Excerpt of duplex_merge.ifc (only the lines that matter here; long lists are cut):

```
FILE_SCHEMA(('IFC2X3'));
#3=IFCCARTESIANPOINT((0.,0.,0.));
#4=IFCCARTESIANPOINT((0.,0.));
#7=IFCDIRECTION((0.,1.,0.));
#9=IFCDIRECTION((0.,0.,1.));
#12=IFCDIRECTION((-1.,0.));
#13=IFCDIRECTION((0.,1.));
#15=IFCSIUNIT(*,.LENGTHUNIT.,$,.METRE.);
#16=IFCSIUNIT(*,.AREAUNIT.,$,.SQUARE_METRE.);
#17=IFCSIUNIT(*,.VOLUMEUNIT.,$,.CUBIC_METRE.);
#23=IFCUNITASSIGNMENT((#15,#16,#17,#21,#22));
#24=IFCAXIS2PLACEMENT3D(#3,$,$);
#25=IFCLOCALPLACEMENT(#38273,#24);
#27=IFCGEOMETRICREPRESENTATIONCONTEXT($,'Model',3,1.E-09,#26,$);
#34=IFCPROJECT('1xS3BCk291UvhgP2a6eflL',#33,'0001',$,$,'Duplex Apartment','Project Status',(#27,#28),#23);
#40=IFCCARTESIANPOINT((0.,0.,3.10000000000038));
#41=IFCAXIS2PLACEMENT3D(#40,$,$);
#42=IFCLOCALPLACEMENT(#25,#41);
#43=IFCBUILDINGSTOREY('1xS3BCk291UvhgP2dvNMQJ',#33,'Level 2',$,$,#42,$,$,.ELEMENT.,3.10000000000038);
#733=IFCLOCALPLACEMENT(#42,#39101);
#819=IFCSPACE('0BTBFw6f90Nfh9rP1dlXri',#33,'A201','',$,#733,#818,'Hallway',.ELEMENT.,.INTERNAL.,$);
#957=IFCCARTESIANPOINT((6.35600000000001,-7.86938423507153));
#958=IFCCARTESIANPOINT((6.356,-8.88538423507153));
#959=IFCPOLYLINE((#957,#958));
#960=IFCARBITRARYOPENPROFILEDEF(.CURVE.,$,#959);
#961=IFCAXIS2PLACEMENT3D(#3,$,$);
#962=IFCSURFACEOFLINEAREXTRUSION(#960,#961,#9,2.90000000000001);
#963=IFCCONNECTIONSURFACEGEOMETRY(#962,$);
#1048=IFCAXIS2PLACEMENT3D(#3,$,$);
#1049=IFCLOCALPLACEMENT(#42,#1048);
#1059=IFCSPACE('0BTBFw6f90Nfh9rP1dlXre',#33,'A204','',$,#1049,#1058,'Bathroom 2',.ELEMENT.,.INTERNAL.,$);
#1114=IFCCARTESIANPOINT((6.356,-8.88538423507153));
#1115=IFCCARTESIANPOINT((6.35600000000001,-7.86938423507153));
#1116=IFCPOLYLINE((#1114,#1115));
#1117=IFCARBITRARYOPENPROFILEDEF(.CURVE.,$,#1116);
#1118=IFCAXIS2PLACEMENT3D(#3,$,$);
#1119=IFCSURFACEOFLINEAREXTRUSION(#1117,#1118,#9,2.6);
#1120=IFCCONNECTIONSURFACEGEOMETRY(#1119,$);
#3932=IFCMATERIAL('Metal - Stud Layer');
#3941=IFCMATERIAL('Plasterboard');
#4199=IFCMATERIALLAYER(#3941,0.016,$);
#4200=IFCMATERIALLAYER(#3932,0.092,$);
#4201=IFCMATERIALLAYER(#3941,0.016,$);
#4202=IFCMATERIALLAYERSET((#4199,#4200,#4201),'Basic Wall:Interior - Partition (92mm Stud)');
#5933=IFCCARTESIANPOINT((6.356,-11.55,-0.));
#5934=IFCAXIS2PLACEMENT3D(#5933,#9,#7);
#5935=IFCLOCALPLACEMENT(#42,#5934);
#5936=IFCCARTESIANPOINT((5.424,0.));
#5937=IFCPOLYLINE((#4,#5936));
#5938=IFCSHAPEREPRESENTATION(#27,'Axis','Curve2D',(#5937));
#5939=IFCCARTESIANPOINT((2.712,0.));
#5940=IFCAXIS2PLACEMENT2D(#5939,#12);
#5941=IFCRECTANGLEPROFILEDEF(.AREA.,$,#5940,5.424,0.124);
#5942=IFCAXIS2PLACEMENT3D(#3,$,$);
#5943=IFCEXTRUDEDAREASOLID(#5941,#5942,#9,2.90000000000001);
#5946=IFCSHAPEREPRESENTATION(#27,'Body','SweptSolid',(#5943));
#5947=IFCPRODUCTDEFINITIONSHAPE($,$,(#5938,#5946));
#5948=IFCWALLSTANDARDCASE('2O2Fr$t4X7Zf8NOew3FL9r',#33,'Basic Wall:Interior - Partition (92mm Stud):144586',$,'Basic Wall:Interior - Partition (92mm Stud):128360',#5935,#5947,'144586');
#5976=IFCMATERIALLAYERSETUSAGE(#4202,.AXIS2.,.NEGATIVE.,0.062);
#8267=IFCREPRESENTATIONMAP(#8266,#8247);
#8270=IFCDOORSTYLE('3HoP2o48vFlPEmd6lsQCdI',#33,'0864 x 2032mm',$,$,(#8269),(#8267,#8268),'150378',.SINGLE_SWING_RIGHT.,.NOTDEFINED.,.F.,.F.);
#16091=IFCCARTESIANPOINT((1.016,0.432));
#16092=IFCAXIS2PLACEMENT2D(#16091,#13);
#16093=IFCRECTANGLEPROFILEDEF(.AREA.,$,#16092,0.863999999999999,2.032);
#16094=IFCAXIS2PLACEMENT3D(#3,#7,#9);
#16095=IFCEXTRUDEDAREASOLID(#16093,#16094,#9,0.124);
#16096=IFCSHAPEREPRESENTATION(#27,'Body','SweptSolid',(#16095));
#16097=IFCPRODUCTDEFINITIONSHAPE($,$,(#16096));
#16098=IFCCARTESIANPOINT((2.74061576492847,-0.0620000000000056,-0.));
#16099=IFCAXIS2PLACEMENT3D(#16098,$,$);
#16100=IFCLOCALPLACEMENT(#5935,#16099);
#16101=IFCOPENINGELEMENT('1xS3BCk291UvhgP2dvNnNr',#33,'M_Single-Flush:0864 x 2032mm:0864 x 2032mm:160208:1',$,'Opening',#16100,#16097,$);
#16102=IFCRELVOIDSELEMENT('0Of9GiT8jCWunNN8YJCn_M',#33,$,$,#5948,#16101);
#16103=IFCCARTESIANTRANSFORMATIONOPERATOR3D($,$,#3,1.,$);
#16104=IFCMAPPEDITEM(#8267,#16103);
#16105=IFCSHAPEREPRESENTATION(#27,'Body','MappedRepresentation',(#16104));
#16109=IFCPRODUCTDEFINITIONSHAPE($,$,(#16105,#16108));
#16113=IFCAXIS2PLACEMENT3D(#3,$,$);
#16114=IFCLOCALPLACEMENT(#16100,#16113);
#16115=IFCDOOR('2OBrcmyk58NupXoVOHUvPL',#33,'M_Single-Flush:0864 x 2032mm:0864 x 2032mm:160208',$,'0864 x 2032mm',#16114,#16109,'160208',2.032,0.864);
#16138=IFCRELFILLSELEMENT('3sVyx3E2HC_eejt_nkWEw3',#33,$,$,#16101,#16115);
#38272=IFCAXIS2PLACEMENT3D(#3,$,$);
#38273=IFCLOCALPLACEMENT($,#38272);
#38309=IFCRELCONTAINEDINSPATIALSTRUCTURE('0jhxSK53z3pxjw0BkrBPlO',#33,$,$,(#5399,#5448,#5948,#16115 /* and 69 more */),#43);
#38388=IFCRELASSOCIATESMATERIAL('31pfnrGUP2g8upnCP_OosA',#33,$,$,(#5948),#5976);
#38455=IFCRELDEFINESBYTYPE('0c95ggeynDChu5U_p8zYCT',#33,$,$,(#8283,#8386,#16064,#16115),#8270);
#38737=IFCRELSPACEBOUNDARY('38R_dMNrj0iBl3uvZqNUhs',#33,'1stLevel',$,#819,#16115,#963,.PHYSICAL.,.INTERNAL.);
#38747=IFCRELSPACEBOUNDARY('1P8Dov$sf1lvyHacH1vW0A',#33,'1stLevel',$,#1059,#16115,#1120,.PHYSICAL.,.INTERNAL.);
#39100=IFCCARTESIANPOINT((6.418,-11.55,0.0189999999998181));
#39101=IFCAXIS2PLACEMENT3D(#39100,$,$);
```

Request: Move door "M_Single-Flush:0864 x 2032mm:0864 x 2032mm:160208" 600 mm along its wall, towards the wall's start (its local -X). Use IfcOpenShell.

```python
import numpy as np
import ifcopenshell
import ifcopenshell.api.geometry
import ifcopenshell.util.placement

model = ifcopenshell.open("duplex_merge.ifc")

door = model.by_id(16115)
opening = door.FillsVoids[0].RelatingOpeningElement
wall = opening.VoidsElements[0].RelatingBuildingElement

wall_matrix = ifcopenshell.util.placement.get_local_placement(wall.ObjectPlacement)
shift = wall_matrix[:3, 0] * -0.6
before = ifcopenshell.util.placement.get_local_placement(door.ObjectPlacement)[:3, 3].copy()

# The door is placed relative to its opening, so it follows when the opening moves.
matrix = ifcopenshell.util.placement.get_local_placement(opening.ObjectPlacement)
matrix[:3, 3] += shift
ifcopenshell.api.geometry.edit_object_placement(
    model, product=opening, matrix=matrix, is_si=False, should_transform_children=True
)

# Space boundary surfaces are stored in each space's coordinates; move them too.
for rel in door.ProvidesBoundaries:
    if not rel.ConnectionGeometry:
        continue
    surface = rel.ConnectionGeometry.SurfaceOnRelatingElement
    space_matrix = ifcopenshell.util.placement.get_local_placement(rel.RelatingSpace.ObjectPlacement)
    point = np.array(surface.Position.Location.Coordinates) + space_matrix[:3, :3].T @ shift
    surface.Position = model.createIfcAxis2Placement3D(
        model.createIfcCartesianPoint(point.tolist()), surface.Position.Axis, surface.Position.RefDirection
    )

after = ifcopenshell.util.placement.get_local_placement(door.ObjectPlacement)[:3, 3]
print("door moved by", (after - before).round(3) + 0.0)

model.write("duplex_merge-out.ifc")
```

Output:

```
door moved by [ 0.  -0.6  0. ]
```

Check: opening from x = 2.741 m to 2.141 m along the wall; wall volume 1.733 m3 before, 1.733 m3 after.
